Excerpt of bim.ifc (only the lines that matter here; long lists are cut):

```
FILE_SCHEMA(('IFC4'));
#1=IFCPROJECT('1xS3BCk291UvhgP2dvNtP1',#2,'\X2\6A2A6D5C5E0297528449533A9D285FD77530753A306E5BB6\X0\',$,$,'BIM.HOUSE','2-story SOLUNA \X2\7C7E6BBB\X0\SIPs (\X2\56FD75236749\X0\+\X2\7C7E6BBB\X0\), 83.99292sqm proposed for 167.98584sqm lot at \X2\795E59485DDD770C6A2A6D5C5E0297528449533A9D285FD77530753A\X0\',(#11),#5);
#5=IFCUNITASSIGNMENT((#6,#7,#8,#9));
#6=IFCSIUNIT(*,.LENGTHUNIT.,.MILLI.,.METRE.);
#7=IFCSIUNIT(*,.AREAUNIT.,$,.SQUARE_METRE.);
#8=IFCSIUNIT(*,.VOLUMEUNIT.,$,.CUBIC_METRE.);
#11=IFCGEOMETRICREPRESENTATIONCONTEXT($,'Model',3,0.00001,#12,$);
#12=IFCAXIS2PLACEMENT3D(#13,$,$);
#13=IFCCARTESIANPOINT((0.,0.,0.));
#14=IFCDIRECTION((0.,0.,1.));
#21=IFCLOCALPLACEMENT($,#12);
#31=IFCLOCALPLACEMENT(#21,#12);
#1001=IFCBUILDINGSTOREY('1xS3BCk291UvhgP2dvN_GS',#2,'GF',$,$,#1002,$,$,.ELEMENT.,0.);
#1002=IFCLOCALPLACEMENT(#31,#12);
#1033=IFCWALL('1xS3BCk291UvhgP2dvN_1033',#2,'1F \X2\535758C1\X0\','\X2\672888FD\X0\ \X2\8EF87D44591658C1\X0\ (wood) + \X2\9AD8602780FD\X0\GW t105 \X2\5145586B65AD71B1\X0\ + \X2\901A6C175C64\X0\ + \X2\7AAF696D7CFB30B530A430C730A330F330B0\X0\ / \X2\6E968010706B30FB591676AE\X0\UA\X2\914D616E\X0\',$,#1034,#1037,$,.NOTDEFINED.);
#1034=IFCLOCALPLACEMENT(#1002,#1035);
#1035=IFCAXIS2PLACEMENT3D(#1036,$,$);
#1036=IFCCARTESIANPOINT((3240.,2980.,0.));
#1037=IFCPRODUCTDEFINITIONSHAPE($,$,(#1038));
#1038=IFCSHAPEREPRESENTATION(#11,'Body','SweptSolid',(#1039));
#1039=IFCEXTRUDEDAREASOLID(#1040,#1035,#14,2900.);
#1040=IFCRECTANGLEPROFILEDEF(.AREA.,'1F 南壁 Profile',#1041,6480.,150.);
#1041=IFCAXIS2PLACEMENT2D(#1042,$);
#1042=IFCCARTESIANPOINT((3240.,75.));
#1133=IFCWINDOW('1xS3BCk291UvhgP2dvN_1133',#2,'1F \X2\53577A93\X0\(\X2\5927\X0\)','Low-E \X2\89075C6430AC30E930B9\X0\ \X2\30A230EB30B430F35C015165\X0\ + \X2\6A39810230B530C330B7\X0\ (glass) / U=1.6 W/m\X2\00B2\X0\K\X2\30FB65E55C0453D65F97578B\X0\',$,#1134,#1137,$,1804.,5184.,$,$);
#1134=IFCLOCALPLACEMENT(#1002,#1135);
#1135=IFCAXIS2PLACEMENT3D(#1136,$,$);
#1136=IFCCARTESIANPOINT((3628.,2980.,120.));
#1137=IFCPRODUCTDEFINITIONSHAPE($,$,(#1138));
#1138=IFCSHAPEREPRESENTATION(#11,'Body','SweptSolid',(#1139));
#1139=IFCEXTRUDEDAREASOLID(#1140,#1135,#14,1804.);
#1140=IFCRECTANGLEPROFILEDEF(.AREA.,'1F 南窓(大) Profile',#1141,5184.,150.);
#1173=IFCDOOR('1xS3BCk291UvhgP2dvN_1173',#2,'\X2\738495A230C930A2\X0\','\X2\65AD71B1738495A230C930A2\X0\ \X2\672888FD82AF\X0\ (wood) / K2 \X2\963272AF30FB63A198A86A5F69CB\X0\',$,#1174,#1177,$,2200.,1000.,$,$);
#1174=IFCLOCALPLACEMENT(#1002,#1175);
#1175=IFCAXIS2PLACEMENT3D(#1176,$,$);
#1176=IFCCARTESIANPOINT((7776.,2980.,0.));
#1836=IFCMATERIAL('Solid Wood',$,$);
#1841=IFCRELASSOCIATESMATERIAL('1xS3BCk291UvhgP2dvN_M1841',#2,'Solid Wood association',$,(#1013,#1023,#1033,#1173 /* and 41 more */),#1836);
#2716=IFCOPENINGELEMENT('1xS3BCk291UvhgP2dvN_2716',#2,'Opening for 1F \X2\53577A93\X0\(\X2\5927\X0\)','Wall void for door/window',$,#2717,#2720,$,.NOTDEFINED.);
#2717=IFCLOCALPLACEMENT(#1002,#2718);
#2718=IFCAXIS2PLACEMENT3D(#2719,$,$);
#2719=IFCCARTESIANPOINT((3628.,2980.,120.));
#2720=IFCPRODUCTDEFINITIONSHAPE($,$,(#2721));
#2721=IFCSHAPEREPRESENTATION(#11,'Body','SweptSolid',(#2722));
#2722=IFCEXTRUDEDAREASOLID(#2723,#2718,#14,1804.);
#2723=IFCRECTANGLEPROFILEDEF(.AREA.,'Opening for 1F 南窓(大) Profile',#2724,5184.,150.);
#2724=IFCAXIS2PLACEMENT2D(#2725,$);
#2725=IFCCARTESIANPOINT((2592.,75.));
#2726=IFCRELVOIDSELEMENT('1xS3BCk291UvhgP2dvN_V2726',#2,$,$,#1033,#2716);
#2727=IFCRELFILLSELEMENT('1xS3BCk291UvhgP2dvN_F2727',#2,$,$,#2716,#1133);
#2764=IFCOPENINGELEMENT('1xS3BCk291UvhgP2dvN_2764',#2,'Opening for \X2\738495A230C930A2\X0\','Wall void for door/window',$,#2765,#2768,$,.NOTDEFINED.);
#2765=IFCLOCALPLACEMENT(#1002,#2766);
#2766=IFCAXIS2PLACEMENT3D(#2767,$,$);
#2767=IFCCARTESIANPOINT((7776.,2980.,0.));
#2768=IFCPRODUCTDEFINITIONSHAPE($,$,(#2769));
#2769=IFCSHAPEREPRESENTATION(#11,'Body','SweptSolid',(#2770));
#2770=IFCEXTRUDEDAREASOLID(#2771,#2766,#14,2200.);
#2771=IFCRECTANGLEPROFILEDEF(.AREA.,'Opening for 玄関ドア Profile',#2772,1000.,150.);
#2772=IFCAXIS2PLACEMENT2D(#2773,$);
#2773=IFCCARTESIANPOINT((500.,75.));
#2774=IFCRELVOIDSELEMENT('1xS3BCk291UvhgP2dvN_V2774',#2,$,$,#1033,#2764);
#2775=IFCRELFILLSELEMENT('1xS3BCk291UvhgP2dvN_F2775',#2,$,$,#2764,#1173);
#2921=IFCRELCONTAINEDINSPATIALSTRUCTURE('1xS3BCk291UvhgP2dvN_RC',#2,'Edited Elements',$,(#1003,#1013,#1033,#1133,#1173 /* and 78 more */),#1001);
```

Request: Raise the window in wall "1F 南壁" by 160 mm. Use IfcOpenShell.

```python
import numpy as np
import ifcopenshell
import ifcopenshell.api.geometry
import ifcopenshell.util.placement
import ifcopenshell.util.unit

model = ifcopenshell.open("bim.ifc")
unit_scale = ifcopenshell.util.unit.calculate_unit_scale(model)

window = model.by_id(1133)
opening = window.FillsVoids[0].RelatingOpeningElement
dz = 160.0

shift = np.array([0.0, 0.0, dz])
# The window is not placed relative to its opening, so move both.
for product in (opening, window):
    matrix = ifcopenshell.util.placement.get_local_placement(product.ObjectPlacement)
    matrix[:3, 3] += shift
    ifcopenshell.api.geometry.edit_object_placement(model, product=product, matrix=matrix, is_si=False)

print(f"moved by {dz * unit_scale:+.3f} m")

model.write("bim-out.ifc")
```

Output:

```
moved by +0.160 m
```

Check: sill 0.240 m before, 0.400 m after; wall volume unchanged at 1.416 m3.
